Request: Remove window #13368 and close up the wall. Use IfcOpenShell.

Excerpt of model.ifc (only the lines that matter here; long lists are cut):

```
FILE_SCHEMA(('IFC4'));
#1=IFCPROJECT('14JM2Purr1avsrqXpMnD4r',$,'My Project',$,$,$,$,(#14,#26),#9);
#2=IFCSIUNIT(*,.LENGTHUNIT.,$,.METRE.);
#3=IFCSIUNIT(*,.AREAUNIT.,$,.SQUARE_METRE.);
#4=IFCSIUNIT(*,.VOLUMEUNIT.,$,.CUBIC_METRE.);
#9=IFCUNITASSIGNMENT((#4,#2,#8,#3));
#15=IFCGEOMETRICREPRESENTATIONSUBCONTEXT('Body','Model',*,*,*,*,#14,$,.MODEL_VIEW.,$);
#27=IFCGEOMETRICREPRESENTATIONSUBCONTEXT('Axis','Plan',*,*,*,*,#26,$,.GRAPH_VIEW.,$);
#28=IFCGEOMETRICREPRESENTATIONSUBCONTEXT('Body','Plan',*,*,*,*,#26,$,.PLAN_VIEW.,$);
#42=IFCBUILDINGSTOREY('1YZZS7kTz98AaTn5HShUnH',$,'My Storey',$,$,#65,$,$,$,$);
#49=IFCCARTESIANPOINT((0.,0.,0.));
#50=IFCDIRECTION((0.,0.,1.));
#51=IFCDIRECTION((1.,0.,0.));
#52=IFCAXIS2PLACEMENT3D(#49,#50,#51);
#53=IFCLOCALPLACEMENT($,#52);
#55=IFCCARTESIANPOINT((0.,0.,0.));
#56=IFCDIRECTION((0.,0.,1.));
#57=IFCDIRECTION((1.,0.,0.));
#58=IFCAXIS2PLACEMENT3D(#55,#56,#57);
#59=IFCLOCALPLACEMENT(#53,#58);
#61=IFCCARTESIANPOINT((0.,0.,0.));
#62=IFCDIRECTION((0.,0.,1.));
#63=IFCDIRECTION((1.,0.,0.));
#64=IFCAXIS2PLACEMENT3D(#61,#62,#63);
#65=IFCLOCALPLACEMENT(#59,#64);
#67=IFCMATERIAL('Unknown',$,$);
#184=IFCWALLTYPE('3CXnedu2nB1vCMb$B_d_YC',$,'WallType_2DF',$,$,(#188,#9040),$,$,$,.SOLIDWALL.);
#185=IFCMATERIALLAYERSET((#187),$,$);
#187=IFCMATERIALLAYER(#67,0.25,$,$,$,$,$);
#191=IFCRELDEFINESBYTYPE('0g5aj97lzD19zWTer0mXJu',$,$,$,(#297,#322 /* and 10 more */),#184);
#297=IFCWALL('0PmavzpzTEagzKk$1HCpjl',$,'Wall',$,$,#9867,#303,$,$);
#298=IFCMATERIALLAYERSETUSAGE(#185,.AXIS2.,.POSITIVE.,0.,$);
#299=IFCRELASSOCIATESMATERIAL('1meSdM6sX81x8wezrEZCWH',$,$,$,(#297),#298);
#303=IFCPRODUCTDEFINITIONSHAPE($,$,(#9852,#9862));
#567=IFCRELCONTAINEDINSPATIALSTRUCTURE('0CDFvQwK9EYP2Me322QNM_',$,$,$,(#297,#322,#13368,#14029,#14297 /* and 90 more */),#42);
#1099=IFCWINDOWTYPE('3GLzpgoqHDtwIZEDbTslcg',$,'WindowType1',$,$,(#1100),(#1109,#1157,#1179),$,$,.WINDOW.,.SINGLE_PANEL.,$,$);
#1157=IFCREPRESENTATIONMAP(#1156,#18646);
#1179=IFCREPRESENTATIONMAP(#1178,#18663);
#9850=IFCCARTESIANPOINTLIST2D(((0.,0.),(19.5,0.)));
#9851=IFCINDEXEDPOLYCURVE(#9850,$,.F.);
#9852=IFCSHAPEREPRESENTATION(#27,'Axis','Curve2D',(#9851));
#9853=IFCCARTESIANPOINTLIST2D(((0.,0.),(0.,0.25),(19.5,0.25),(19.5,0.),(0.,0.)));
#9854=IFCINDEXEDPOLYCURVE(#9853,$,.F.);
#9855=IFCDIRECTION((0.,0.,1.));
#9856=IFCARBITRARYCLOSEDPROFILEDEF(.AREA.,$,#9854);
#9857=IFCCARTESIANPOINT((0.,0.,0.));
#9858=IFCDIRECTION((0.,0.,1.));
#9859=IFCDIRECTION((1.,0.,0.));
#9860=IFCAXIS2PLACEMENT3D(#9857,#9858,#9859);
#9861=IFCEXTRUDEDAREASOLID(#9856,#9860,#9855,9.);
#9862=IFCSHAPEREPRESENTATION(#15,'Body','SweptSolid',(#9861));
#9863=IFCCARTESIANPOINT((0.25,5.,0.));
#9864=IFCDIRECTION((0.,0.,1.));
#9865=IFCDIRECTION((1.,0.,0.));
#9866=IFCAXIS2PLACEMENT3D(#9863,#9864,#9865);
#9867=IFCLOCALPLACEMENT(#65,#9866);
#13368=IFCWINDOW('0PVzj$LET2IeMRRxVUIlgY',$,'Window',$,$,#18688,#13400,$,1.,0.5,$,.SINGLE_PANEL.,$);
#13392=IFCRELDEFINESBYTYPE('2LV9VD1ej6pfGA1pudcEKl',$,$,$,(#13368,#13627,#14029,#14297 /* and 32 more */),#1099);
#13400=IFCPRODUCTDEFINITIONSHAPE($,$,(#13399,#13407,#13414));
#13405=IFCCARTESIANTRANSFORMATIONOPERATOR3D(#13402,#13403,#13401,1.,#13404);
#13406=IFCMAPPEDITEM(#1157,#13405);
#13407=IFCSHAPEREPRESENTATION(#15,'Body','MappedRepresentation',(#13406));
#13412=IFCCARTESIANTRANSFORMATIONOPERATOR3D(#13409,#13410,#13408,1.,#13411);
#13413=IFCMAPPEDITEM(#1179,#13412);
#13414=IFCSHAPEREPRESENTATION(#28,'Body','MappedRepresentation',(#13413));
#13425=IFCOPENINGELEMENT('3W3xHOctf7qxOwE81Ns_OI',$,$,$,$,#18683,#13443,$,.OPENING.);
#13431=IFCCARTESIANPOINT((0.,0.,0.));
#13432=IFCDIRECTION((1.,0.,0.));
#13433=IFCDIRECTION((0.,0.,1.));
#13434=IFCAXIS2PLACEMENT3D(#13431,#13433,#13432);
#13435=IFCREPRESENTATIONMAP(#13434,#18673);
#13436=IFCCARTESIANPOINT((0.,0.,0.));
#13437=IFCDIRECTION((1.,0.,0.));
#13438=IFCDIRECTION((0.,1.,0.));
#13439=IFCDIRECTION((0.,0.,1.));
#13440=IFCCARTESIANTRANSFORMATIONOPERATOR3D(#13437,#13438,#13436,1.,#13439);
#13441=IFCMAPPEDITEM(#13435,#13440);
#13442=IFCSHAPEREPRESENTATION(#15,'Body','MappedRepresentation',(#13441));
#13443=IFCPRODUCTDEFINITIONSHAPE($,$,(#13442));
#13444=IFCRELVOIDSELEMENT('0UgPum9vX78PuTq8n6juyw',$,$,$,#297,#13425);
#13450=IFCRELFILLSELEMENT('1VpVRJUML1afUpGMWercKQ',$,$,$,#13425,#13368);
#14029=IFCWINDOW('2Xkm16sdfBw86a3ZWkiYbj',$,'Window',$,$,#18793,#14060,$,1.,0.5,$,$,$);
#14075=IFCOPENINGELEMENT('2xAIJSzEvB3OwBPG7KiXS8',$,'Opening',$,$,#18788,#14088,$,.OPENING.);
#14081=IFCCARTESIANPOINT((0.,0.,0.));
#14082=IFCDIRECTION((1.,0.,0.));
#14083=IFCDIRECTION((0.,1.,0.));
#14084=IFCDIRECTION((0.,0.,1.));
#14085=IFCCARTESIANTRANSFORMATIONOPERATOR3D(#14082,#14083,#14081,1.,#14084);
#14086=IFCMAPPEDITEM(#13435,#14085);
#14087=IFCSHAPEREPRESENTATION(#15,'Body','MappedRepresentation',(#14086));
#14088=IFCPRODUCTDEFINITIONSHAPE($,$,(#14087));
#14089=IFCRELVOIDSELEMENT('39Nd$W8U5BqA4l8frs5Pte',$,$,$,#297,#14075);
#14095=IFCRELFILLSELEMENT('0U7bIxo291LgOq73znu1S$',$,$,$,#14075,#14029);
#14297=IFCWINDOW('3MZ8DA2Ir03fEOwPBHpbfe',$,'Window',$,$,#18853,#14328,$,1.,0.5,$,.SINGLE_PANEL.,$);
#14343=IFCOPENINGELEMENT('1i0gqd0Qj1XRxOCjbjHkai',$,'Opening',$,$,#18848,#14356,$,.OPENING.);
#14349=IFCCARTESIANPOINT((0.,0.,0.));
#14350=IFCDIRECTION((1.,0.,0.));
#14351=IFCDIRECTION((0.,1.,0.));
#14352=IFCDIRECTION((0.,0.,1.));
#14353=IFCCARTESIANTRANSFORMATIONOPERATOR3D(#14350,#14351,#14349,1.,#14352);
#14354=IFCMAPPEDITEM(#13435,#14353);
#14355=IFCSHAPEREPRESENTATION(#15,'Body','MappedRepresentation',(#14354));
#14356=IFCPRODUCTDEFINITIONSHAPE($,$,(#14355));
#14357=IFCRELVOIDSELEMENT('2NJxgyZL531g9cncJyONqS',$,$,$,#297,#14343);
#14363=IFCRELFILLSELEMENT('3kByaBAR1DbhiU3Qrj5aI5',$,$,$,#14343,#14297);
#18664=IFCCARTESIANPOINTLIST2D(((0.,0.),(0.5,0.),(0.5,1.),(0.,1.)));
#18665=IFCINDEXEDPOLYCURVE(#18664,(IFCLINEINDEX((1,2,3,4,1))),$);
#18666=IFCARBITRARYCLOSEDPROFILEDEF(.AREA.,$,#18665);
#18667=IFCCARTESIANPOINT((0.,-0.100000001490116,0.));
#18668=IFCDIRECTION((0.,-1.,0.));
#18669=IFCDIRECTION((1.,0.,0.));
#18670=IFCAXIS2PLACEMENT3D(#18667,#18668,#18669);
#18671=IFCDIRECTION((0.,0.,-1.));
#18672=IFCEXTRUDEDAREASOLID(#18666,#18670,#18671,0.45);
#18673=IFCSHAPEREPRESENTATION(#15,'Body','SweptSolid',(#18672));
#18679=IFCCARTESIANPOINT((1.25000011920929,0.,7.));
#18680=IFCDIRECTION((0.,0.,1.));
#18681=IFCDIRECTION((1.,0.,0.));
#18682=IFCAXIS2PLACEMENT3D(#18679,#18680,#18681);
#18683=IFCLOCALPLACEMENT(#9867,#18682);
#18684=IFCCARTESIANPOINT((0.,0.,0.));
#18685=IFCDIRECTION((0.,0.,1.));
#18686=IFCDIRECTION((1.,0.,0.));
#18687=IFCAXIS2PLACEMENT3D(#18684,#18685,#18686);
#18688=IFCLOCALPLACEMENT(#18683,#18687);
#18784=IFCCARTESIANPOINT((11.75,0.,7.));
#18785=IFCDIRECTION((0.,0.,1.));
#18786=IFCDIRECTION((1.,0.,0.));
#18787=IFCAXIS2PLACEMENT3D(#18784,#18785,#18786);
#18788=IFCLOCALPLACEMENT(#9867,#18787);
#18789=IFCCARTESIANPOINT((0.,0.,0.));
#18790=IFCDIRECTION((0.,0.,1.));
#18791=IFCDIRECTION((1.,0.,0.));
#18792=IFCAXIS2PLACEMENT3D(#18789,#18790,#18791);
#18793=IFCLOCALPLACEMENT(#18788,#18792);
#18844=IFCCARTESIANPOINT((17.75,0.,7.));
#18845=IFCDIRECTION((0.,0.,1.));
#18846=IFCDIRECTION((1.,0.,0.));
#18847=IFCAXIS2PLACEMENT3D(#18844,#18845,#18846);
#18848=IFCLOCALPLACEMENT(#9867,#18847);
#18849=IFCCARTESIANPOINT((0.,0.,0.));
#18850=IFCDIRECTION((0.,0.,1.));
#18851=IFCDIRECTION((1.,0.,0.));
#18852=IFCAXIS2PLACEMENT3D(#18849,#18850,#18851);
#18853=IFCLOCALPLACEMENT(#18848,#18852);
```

```python
import ifcopenshell
import ifcopenshell.api.feature
import ifcopenshell.api.root
import ifcopenshell.geom
import ifcopenshell.util.shape

model = ifcopenshell.open("model.ifc")
settings = ifcopenshell.geom.settings()


def volume(element):
    """Net volume in cubic metres, openings subtracted."""
    shape = ifcopenshell.geom.create_shape(settings, element)
    return ifcopenshell.util.shape.get_volume(shape.geometry)


window = model.by_guid("0PVzj$LET2IeMRRxVUIlgY")
opening = window.FillsVoids[0].RelatingOpeningElement
wall = opening.VoidsElements[0].RelatingBuildingElement
before = volume(wall)

ifcopenshell.api.root.remove_product(model, product=window)
ifcopenshell.api.feature.remove_feature(model, feature=opening)

after = volume(wall)

print(f"wall volume {before:.3f} -> {after:.3f} m3")

model.write("model-out.ifc")
```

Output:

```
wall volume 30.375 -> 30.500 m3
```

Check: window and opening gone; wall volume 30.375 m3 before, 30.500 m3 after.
